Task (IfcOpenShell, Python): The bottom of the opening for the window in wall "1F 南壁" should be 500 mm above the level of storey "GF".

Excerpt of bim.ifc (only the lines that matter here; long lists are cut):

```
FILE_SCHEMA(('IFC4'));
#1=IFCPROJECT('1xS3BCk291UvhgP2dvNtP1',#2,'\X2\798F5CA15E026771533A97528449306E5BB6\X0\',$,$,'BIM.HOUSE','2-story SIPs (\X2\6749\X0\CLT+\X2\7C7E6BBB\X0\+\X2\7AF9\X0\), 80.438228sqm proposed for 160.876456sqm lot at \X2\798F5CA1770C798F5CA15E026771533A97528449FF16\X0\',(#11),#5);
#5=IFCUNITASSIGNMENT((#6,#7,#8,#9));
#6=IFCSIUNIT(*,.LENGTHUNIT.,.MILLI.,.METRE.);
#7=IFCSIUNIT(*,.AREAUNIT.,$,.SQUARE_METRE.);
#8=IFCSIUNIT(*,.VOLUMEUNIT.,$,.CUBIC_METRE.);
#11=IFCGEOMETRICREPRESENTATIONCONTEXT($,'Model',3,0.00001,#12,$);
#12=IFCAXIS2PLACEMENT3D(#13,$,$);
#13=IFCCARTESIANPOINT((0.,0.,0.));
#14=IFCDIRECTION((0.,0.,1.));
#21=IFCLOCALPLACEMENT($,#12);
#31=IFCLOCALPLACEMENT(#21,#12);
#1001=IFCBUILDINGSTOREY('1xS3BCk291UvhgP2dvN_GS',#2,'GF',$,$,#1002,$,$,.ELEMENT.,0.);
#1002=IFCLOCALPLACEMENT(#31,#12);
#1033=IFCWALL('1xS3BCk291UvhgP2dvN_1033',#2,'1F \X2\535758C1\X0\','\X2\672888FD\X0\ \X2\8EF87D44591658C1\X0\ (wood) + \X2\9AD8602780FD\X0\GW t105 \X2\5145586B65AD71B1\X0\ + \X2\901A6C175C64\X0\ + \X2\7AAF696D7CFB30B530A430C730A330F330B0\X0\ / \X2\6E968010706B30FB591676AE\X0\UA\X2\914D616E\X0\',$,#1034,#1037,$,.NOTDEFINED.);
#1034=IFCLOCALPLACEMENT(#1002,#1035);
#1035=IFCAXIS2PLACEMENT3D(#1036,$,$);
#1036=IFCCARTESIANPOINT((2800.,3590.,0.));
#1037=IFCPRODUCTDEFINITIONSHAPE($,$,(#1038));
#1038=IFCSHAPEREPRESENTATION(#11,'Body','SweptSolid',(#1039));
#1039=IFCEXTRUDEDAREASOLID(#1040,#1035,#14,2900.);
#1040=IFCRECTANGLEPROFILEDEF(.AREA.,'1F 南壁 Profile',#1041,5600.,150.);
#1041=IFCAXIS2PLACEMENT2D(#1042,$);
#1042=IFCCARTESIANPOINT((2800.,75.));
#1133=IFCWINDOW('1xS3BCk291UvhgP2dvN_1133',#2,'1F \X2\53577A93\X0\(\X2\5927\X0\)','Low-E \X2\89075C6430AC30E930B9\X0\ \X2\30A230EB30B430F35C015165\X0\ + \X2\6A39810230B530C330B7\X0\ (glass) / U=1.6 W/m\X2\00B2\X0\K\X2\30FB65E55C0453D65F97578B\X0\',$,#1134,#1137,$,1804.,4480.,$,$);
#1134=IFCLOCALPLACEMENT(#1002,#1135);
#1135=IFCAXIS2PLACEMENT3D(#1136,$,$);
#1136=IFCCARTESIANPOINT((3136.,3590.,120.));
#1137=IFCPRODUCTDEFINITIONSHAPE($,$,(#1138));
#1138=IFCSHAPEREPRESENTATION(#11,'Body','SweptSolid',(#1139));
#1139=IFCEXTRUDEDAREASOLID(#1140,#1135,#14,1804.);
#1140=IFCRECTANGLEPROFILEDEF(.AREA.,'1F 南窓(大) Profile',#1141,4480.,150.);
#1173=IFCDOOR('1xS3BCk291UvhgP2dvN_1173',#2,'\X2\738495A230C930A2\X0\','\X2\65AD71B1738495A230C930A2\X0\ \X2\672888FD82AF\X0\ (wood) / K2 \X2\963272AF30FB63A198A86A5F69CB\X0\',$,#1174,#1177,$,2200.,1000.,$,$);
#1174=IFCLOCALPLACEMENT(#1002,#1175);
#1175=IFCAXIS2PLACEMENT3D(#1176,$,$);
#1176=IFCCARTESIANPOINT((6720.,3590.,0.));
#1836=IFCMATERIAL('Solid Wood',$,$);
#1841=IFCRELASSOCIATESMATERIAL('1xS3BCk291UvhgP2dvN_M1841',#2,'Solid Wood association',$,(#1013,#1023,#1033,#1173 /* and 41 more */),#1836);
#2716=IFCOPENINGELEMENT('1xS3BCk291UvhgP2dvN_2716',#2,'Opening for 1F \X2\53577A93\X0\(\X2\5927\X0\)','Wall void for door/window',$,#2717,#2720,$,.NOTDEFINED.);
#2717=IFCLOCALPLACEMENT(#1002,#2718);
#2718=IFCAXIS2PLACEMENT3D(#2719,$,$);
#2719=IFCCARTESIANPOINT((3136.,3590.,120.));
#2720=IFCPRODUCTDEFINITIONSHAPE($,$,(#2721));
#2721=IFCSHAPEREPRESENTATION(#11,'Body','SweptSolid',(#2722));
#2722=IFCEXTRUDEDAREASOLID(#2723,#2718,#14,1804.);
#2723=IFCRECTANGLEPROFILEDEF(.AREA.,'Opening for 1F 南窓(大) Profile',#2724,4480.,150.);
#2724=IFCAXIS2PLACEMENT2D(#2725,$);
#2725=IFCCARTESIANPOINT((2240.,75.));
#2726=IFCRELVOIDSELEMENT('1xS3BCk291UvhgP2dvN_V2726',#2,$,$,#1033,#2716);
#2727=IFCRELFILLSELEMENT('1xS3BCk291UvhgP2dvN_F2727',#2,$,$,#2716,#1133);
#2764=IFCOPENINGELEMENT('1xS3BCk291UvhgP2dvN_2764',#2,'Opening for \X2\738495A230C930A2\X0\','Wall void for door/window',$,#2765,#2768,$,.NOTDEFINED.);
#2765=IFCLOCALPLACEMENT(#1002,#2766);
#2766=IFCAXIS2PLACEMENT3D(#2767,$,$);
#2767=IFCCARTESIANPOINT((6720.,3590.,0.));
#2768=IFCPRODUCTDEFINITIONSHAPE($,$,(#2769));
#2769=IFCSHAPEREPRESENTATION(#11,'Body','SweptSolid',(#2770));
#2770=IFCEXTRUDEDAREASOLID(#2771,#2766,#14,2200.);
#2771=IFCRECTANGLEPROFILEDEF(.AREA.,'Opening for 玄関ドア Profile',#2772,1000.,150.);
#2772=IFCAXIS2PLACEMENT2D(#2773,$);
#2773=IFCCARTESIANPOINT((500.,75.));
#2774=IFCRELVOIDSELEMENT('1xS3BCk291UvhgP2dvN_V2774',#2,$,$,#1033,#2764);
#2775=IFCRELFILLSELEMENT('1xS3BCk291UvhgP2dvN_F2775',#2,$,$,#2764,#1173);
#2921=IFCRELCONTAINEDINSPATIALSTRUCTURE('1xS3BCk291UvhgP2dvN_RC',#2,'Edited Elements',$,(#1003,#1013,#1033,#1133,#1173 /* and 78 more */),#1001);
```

```python
import numpy as np
import ifcopenshell
import ifcopenshell.api.geometry
import ifcopenshell.geom
import ifcopenshell.util.element
import ifcopenshell.util.placement
import ifcopenshell.util.shape
import ifcopenshell.util.unit

model = ifcopenshell.open("bim.ifc")
unit_scale = ifcopenshell.util.unit.calculate_unit_scale(model)

window = model.by_guid("1xS3BCk291UvhgP2dvN_1133")
opening = window.FillsVoids[0].RelatingOpeningElement
storey = ifcopenshell.util.element.get_container(window, ifc_class="IfcBuildingStorey")
level = ifcopenshell.util.placement.get_local_placement(storey.ObjectPlacement)[2, 3]

# The opening's origin need not be at the sill, so measure its lowest point.
shape = ifcopenshell.geom.create_shape(ifcopenshell.geom.settings(), opening)
bottom = ifcopenshell.util.shape.get_shape_bottom_elevation(shape, shape.geometry) / unit_scale
dz = level + 0.5 / unit_scale - bottom

shift = np.array([0.0, 0.0, dz])
# The window is not placed relative to its opening, so move both.
for product in (opening, window):
    matrix = ifcopenshell.util.placement.get_local_placement(product.ObjectPlacement)
    matrix[:3, 3] += shift
    ifcopenshell.api.geometry.edit_object_placement(model, product=product, matrix=matrix, is_si=False)

print(f"moved by {dz * unit_scale:+.3f} m")

model.write("bim_edited.ifc")
```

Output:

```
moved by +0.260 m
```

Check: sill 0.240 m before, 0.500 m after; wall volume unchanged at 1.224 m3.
